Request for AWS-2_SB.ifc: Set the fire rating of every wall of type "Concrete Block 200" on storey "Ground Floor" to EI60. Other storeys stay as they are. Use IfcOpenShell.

First a look at what the model holds.

```python
import ifcopenshell
import ifcopenshell.util.element

model = ifcopenshell.open("AWS-2_SB.ifc")
print(model.schema)
storey = next(s for s in model.by_type("IfcBuildingStorey") if s.Name == "Ground Floor")
walls = [e for e in ifcopenshell.util.element.get_decomposition(storey) if e.is_a("IfcWall")]
seen = {}
for e in walls:
    element_type = ifcopenshell.util.element.get_type(e)
    key = (element_type.Name if element_type != e and element_type else None, ifcopenshell.util.element.get_pset(e, "Pset_WallCommon", "FireRating"))
    seen[key] = seen.get(key, 0) + 1
for (name, value), count in sorted(seen.items(), key=str):
    print(count, "x", name, "|", value)
```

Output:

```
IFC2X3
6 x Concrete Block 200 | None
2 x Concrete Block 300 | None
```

```python
import ifcopenshell
import ifcopenshell.api.pset
import ifcopenshell.util.element

model = ifcopenshell.open("AWS-2_SB.ifc")

storey = next(s for s in model.by_type("IfcBuildingStorey") if s.Name == "Ground Floor")
walls = [e for e in ifcopenshell.util.element.get_decomposition(storey) if e.is_a("IfcWall")]

count = 0
for e in walls:
    element_type = ifcopenshell.util.element.get_type(e)
    if element_type in (None, e) or element_type.Name != "Concrete Block 200":
        continue
    # add_pset returns the element's existing set when there is one.
    pset = ifcopenshell.api.pset.add_pset(model, product=e, name="Pset_WallCommon")
    ifcopenshell.api.pset.edit_pset(model, pset=pset, properties={"FireRating": "EI60"})
    count += 1

print(count, "walls updated")

model.write("AWS-2_SB-out.ifc")
```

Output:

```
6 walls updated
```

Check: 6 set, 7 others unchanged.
